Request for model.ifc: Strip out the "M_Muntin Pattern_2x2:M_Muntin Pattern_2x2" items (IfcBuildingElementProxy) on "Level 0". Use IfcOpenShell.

First a look at what the model holds.

```python
import ifcopenshell
import ifcopenshell.util.element

model = ifcopenshell.open("model.ifc")
print(model.schema)
storey = next(s for s in model.by_type("IfcBuildingStorey") if s.Name == "Level 0")
proxies = [e for e in ifcopenshell.util.element.get_decomposition(storey) if e.is_a("IfcBuildingElementProxy")]
seen = {}
for e in proxies:
    element_type = ifcopenshell.util.element.get_type(e)
    name = element_type.Name if element_type not in (None, e) else None
    seen[name] = seen.get(name, 0) + 1
for name, count in sorted(seen.items(), key=str):
    print(count, "x", name)
```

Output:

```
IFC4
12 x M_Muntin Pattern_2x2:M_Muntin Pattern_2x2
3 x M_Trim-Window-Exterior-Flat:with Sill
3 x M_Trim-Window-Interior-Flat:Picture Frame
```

```python
import ifcopenshell
import ifcopenshell.api.root
import ifcopenshell.util.element

model = ifcopenshell.open("model.ifc")

storey = next(s for s in model.by_type("IfcBuildingStorey") if s.Name == "Level 0")
proxies = [e for e in ifcopenshell.util.element.get_decomposition(storey) if e.is_a("IfcBuildingElementProxy")]
targets = [e for e in proxies if (t := ifcopenshell.util.element.get_type(e)) not in (None, e) and t.Name == "M_Muntin Pattern_2x2:M_Muntin Pattern_2x2"]

for e in targets:
    ifcopenshell.api.root.remove_product(model, product=e)
print(len(targets), "removed")

model.write("model_rev.ifc")
```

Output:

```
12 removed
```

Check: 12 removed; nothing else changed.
